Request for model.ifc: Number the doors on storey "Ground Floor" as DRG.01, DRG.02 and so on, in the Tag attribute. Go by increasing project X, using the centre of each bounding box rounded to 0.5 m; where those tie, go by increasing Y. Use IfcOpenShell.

First a look at what the model holds.

```python
import ifcopenshell
import ifcopenshell.util.element
import ifcopenshell.util.placement

model = ifcopenshell.open("model.ifc")
print(model.schema)
storey = next(s for s in model.by_type("IfcBuildingStorey") if s.Name == "Ground Floor")
doors = [e for e in ifcopenshell.util.element.get_decomposition(storey) if e.is_a("IfcDoor")]
for e in sorted(doors, key=lambda e: e.id()):
    origin = ifcopenshell.util.placement.get_local_placement(e.ObjectPlacement)[:3, 3]
    print(e.id(), e.Tag, e.Name, origin.round(2) + 0.0, sep=" | ")
```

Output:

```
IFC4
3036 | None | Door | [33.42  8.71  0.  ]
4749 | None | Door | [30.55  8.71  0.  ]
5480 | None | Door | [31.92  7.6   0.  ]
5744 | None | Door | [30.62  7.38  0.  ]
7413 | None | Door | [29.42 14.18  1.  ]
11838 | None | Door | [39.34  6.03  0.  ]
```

```python
import ifcopenshell
import ifcopenshell.geom
import ifcopenshell.util.element
import ifcopenshell.util.shape

model = ifcopenshell.open("model.ifc")
settings = ifcopenshell.geom.settings()
settings.set("use-world-coords", True)


def centre(element):
    shape = ifcopenshell.geom.create_shape(settings, element)
    return ifcopenshell.util.shape.get_bbox_centroid(shape.geometry)


storey = next(s for s in model.by_type("IfcBuildingStorey") if s.Name == "Ground Floor")
doors = [e for e in ifcopenshell.util.element.get_decomposition(storey) if e.is_a("IfcDoor")]

# Insertion points can sit at a corner or the storey origin, so sort by the geometry (in metres).
centres = {e: centre(e) for e in doors}
doors.sort(key=lambda e: (round(centres[e][0] / 0.5), centres[e][1]))

for i, e in enumerate(doors, start=1):
    number = f"DRG.{i:02d}"
    e.Tag = number
    print(e.id(), number)

model.write("model_v2.ifc")
```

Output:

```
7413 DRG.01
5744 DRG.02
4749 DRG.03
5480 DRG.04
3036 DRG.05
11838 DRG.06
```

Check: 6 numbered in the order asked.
